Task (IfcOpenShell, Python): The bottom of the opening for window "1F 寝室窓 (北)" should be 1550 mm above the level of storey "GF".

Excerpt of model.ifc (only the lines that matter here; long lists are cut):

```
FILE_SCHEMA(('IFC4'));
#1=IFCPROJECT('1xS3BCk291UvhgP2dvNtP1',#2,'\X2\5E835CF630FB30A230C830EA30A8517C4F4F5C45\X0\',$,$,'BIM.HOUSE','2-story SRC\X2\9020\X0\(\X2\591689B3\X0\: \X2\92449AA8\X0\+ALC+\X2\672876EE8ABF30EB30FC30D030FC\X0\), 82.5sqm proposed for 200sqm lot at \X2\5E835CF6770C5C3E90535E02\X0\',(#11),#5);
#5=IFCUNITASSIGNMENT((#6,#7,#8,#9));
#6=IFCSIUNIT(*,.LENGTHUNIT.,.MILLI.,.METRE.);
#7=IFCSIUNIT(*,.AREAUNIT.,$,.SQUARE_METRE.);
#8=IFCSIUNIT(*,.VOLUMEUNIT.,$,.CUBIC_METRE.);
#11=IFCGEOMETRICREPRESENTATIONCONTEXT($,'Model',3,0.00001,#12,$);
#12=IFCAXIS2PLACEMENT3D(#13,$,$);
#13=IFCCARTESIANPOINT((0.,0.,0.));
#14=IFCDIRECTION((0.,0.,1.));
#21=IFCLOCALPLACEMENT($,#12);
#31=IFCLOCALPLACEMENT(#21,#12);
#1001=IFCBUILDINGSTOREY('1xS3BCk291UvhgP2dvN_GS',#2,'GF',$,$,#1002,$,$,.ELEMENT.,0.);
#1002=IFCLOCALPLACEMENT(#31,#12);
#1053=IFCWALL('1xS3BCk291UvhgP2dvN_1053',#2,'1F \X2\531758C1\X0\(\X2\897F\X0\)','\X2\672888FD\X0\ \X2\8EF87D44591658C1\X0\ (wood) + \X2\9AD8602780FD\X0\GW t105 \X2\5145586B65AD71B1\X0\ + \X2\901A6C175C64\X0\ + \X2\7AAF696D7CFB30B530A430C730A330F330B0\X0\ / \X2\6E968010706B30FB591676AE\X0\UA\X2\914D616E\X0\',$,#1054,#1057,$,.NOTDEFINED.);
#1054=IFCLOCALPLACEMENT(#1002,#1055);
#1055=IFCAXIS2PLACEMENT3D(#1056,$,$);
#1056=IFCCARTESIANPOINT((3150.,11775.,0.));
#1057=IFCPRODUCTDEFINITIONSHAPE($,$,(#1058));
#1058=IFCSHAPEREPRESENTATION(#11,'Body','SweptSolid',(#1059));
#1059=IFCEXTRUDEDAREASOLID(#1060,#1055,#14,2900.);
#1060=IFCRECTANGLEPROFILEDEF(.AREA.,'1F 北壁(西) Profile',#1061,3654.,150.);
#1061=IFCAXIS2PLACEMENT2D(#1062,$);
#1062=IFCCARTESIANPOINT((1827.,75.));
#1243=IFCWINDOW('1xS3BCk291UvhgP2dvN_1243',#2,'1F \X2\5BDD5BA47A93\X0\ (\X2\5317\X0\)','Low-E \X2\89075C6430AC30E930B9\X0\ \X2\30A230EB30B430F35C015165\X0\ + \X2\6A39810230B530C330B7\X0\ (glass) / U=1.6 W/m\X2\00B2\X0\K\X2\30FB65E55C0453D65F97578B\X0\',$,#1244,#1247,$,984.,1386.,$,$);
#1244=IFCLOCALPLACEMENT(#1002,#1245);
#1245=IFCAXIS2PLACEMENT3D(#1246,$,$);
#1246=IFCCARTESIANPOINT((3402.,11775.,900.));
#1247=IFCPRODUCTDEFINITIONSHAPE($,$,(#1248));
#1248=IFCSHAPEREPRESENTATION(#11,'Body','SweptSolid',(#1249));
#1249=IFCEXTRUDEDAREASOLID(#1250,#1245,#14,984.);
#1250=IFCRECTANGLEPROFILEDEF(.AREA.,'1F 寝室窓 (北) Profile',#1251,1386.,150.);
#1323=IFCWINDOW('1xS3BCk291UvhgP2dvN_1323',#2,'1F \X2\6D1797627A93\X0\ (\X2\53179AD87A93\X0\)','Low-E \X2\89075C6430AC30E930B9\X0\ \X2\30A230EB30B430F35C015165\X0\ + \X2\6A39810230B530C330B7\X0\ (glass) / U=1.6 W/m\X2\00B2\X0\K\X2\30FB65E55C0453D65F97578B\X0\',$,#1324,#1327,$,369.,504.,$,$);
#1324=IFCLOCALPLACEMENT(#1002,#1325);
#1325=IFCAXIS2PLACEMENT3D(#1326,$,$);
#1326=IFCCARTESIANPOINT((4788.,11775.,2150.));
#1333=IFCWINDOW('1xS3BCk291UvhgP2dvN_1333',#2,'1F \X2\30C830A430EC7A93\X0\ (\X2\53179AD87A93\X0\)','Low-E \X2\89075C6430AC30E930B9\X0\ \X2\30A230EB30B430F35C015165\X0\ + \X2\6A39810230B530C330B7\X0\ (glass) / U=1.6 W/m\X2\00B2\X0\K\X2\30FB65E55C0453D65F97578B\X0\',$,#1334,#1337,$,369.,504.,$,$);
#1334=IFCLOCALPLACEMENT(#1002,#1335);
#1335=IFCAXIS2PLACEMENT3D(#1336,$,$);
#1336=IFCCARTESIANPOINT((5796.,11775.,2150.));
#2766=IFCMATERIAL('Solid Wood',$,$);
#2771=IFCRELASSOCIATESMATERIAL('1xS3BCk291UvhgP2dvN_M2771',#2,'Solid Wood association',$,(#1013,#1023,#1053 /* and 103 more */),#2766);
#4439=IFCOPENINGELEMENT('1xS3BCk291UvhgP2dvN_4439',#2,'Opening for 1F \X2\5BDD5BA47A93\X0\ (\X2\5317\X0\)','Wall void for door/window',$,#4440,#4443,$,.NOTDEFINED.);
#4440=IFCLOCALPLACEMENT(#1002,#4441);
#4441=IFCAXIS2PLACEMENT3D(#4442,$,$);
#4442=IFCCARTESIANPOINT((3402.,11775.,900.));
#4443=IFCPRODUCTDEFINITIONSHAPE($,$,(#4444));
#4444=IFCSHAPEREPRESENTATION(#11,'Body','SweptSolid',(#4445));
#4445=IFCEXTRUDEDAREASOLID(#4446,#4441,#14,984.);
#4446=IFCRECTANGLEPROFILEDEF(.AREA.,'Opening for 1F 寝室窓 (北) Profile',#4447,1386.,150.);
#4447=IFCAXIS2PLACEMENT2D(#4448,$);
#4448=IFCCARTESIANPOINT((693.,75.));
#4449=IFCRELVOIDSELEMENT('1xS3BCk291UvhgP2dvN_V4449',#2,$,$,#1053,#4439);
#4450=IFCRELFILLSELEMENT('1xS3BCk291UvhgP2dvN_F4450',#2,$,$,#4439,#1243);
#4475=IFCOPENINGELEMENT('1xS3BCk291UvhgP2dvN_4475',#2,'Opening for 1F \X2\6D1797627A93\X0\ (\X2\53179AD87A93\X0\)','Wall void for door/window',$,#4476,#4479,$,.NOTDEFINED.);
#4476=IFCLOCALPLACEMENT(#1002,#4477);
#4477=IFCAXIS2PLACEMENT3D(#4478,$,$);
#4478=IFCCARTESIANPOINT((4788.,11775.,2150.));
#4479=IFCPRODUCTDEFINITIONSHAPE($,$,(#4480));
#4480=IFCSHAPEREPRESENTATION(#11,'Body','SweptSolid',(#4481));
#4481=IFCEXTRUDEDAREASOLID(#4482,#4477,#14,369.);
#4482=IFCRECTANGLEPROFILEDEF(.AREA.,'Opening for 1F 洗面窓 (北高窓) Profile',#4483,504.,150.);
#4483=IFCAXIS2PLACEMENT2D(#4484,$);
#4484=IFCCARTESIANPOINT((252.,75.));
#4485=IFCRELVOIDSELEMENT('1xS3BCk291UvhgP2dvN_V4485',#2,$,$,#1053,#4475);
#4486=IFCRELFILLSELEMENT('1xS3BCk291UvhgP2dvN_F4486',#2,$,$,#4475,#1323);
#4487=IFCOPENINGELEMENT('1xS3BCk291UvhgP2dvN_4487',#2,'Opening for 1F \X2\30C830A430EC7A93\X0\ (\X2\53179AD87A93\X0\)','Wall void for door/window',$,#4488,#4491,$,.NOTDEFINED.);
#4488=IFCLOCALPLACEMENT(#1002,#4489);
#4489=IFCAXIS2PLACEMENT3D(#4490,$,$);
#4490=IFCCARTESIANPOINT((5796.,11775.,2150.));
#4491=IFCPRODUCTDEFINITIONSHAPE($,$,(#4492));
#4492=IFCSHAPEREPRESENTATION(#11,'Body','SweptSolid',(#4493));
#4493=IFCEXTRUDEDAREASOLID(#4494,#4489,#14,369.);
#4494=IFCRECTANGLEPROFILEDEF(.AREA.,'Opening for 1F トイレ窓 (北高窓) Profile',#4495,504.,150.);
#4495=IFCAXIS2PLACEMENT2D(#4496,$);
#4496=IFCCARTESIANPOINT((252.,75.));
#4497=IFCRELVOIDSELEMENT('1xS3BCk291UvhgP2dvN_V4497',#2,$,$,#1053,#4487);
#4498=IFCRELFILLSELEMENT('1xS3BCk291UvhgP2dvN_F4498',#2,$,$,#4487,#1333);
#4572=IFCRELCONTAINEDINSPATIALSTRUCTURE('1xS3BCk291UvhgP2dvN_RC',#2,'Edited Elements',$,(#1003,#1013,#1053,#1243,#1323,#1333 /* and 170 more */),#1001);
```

```python
import numpy as np
import ifcopenshell
import ifcopenshell.api.geometry
import ifcopenshell.geom
import ifcopenshell.util.element
import ifcopenshell.util.placement
import ifcopenshell.util.shape
import ifcopenshell.util.unit

model = ifcopenshell.open("model.ifc")
unit_scale = ifcopenshell.util.unit.calculate_unit_scale(model)

window = model.by_guid("1xS3BCk291UvhgP2dvN_1243")
opening = window.FillsVoids[0].RelatingOpeningElement
storey = ifcopenshell.util.element.get_container(window, ifc_class="IfcBuildingStorey")
level = ifcopenshell.util.placement.get_local_placement(storey.ObjectPlacement)[2, 3]

# The opening's origin need not be at the sill, so measure its lowest point.
shape = ifcopenshell.geom.create_shape(ifcopenshell.geom.settings(), opening)
bottom = ifcopenshell.util.shape.get_shape_bottom_elevation(shape, shape.geometry) / unit_scale
dz = level + 1.55 / unit_scale - bottom

shift = np.array([0.0, 0.0, dz])
# The window is not placed relative to its opening, so move both.
for product in (opening, window):
    matrix = ifcopenshell.util.placement.get_local_placement(product.ObjectPlacement)
    matrix[:3, 3] += shift
    ifcopenshell.api.geometry.edit_object_placement(model, product=product, matrix=matrix, is_si=False)

print(f"moved by {dz * unit_scale:+.3f} m")

model.write("model_rev.ifc")
```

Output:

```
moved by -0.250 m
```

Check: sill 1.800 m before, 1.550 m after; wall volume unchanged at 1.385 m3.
